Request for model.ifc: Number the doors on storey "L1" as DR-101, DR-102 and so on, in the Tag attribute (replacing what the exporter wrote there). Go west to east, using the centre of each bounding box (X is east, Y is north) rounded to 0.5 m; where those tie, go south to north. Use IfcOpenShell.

First a look at what the model holds.

```python
import ifcopenshell
import ifcopenshell.util.element
import ifcopenshell.util.placement

model = ifcopenshell.open("model.ifc")
print(model.schema)
storey = next(s for s in model.by_type("IfcBuildingStorey") if s.Name == "L1")
doors = [e for e in ifcopenshell.util.element.get_decomposition(storey) if e.is_a("IfcDoor")]
for e in sorted(doors, key=lambda e: e.id()):
    origin = ifcopenshell.util.placement.get_local_placement(e.ObjectPlacement)[:3, 3]
    print(e.id(), e.Tag, e.Name, origin.round(2) + 0.0, sep=" | ")
```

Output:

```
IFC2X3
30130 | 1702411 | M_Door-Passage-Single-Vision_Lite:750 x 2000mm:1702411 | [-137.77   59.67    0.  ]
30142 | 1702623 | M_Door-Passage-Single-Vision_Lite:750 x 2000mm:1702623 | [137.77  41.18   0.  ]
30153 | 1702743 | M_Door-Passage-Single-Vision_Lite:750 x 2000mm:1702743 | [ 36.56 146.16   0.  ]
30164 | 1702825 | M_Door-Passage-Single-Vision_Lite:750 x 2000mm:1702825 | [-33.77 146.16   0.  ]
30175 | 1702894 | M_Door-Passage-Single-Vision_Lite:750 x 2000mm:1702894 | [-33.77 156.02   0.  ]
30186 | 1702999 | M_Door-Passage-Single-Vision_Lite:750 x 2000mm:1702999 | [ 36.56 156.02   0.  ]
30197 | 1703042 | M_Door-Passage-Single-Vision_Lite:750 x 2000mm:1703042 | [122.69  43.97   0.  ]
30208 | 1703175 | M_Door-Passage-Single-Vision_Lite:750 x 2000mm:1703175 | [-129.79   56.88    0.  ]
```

```python
import ifcopenshell
import ifcopenshell.geom
import ifcopenshell.util.element
import ifcopenshell.util.shape

model = ifcopenshell.open("model.ifc")
settings = ifcopenshell.geom.settings()
settings.set("use-world-coords", True)


def centre(element):
    shape = ifcopenshell.geom.create_shape(settings, element)
    return ifcopenshell.util.shape.get_bbox_centroid(shape.geometry)


storey = next(s for s in model.by_type("IfcBuildingStorey") if s.Name == "L1")
doors = [e for e in ifcopenshell.util.element.get_decomposition(storey) if e.is_a("IfcDoor")]

# Insertion points can sit at a corner or the storey origin, so sort by the geometry (in metres).
centres = {e: centre(e) for e in doors}
doors.sort(key=lambda e: (round(centres[e][0] / 0.5), centres[e][1]))

for i, e in enumerate(doors, start=1):
    number = f"DR-1{i:02d}"
    e.Tag = number
    print(e.id(), number)

model.write("model_v2.ifc")
```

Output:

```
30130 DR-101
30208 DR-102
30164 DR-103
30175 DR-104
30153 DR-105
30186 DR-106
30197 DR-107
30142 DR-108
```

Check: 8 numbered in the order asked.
